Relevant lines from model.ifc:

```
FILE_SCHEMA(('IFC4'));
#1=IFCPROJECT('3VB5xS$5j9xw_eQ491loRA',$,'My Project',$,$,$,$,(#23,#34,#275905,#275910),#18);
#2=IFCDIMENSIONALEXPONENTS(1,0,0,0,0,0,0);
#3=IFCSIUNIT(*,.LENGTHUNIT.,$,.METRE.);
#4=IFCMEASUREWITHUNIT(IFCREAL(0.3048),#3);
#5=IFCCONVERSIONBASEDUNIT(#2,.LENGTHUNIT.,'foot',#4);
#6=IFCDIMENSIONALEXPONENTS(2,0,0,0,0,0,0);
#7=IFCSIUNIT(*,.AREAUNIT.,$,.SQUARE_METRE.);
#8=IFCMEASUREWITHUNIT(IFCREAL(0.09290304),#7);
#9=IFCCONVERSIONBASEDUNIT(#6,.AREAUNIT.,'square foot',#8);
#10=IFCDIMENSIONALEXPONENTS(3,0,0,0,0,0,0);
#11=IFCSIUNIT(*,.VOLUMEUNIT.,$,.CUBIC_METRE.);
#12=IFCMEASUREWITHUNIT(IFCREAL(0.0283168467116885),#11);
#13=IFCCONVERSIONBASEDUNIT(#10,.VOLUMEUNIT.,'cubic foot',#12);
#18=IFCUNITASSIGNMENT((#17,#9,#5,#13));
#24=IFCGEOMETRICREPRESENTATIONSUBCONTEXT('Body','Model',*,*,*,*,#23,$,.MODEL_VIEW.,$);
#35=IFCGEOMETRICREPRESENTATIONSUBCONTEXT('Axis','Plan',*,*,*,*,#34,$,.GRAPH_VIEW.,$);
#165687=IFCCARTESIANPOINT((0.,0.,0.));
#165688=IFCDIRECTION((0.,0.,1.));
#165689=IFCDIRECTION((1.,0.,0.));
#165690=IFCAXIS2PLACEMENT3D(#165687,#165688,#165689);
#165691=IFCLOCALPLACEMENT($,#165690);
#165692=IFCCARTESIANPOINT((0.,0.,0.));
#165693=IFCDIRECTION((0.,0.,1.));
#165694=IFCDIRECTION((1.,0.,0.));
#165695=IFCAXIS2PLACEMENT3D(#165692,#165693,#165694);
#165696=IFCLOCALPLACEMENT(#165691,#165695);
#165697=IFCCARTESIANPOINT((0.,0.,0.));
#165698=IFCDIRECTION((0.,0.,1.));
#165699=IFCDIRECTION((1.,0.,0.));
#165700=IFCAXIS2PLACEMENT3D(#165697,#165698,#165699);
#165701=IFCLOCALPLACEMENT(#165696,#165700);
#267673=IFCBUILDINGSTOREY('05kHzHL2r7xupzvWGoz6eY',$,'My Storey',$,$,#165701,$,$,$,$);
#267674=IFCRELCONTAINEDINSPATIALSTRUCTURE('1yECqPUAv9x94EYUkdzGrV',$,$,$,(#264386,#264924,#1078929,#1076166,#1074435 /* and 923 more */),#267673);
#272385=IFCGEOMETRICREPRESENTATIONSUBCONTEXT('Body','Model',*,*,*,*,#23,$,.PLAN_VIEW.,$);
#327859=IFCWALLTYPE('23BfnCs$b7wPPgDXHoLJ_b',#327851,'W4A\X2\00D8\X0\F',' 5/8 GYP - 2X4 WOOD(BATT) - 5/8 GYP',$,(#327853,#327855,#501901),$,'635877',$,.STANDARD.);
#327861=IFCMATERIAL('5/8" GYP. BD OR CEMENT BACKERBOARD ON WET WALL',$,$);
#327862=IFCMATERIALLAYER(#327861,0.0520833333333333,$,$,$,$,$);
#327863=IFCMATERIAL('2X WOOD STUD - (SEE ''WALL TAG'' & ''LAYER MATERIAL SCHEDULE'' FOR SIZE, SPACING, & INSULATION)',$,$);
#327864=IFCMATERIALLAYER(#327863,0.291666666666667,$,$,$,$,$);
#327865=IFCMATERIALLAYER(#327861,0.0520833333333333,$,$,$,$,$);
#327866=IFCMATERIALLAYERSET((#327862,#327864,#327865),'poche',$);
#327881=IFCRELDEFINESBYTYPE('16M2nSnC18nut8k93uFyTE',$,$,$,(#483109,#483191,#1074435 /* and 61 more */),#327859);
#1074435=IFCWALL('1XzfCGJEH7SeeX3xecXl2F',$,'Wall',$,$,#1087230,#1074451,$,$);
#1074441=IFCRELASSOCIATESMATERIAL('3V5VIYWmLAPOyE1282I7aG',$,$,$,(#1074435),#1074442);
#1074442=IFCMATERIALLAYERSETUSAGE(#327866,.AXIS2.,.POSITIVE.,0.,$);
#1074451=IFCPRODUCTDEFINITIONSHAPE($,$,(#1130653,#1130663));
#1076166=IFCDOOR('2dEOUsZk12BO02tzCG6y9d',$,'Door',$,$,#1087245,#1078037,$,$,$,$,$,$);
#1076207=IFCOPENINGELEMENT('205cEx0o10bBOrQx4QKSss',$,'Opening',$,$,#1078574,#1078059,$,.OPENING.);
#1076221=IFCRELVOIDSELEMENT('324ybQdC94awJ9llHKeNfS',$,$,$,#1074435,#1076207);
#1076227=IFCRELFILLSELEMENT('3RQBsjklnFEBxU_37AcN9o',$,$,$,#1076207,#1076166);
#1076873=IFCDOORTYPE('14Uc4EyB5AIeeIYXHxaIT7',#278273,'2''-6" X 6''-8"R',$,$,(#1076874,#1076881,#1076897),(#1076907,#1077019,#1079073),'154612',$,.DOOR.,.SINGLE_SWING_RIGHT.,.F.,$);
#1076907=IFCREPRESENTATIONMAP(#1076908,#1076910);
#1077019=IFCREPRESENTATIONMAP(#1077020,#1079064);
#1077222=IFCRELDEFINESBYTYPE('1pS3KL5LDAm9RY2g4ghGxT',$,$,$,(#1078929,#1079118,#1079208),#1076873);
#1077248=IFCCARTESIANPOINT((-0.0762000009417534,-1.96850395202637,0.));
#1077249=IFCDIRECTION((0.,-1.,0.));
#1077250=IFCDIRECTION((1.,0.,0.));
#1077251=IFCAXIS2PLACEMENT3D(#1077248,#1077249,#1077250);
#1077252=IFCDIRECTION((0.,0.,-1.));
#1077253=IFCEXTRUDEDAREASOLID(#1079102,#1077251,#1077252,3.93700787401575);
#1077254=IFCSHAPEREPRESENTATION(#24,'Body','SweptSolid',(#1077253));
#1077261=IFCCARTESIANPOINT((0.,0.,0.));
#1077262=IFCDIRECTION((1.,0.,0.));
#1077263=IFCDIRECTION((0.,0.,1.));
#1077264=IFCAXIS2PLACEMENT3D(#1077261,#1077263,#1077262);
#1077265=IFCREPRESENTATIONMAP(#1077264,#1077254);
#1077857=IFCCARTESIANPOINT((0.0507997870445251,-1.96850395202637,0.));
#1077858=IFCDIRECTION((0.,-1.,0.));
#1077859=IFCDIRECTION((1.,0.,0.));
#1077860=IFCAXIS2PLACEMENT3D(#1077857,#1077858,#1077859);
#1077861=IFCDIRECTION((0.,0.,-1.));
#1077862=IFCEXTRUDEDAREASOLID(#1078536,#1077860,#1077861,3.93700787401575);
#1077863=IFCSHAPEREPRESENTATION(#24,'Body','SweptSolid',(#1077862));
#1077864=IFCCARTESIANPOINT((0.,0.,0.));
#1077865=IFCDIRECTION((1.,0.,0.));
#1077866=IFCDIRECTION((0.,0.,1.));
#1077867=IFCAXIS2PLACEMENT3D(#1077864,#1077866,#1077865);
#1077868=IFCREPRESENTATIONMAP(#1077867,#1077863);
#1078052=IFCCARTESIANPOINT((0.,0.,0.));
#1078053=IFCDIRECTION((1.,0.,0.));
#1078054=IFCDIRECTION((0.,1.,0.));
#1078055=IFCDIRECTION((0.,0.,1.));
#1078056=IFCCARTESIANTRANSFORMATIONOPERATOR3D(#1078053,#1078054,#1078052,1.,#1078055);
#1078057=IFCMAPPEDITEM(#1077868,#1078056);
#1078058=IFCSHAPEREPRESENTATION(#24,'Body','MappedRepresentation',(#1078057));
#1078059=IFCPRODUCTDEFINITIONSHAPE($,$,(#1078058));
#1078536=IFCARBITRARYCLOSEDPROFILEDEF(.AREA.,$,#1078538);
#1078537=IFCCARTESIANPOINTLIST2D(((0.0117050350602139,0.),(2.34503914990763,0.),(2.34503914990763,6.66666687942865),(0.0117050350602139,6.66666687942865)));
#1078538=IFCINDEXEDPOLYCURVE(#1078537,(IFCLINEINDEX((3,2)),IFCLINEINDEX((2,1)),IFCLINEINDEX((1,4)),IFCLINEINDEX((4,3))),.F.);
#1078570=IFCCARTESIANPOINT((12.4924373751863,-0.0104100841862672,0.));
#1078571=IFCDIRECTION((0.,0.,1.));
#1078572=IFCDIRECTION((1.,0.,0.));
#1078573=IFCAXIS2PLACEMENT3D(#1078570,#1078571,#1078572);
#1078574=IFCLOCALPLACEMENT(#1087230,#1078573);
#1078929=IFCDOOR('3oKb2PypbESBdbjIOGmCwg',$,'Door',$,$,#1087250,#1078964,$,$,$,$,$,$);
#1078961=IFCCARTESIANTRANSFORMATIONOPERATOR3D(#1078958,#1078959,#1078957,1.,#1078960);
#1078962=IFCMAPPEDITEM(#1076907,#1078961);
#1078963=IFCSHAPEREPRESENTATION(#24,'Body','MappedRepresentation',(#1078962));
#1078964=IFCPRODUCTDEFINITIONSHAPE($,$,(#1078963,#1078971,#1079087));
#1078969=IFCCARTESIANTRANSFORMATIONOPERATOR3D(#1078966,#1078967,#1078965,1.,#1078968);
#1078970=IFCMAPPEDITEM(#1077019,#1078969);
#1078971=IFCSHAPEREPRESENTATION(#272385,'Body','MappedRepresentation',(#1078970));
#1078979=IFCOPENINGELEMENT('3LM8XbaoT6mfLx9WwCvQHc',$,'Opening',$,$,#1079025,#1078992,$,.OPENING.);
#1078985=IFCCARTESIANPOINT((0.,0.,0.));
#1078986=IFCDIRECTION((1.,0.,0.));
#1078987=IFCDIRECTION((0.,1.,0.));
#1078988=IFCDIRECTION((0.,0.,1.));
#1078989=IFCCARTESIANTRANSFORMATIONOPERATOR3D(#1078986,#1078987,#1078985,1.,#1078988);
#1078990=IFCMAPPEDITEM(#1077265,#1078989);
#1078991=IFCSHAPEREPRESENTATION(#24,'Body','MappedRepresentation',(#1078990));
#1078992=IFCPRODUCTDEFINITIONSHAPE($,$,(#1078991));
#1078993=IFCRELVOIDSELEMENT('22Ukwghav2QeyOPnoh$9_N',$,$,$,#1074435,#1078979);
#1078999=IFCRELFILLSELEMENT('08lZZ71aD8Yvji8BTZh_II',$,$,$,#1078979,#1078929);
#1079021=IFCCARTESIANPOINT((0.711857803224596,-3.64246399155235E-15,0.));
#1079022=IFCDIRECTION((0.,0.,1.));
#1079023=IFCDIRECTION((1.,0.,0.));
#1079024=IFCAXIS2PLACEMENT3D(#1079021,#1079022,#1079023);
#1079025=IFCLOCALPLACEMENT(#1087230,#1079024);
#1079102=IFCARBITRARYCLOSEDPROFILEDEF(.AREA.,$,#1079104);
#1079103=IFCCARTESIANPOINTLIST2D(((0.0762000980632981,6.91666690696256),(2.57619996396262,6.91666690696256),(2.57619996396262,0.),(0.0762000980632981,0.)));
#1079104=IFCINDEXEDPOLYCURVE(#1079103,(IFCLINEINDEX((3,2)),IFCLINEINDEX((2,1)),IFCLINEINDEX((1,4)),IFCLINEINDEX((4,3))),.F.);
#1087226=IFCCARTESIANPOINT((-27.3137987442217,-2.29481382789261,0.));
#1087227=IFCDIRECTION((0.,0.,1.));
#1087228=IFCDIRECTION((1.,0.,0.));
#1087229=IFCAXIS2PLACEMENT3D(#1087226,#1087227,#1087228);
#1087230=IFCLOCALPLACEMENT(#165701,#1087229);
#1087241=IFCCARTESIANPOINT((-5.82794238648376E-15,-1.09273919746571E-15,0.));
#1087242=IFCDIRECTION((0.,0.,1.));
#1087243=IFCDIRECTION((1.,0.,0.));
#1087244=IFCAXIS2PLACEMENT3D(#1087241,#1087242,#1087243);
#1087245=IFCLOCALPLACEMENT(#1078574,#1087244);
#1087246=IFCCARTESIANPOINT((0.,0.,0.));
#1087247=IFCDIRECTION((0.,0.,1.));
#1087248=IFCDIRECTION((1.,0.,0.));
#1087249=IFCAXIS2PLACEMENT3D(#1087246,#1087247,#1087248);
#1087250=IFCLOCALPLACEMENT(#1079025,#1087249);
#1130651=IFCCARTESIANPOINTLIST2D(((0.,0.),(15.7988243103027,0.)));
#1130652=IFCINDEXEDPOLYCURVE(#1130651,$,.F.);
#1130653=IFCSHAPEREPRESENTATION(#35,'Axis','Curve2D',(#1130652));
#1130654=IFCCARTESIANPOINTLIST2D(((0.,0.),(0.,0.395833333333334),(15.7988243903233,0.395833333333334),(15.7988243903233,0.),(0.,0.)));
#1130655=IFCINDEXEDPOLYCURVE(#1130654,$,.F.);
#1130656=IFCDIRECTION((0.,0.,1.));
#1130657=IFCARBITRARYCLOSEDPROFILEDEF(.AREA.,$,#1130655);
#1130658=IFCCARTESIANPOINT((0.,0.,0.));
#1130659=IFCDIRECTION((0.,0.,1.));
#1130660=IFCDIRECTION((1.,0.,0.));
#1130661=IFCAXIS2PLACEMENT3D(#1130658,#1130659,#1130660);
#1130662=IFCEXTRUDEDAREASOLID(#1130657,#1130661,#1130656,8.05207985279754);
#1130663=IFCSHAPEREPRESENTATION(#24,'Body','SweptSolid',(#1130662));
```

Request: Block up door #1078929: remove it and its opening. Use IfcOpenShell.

```python
import ifcopenshell
import ifcopenshell.api.feature
import ifcopenshell.api.root
import ifcopenshell.geom
import ifcopenshell.util.shape

model = ifcopenshell.open("model.ifc")
settings = ifcopenshell.geom.settings()


def volume(element):
    """Net volume in cubic metres, openings subtracted."""
    shape = ifcopenshell.geom.create_shape(settings, element)
    return ifcopenshell.util.shape.get_volume(shape.geometry)


door = model.by_guid("3oKb2PypbESBdbjIOGmCwg")
opening = door.FillsVoids[0].RelatingOpeningElement
wall = opening.VoidsElements[0].RelatingBuildingElement
before = volume(wall)

ifcopenshell.api.root.remove_product(model, product=door)
ifcopenshell.api.feature.remove_feature(model, feature=opening)

after = volume(wall)

print(f"wall volume {before:.3f} -> {after:.3f} m3")

model.write("model_v2.ifc")
```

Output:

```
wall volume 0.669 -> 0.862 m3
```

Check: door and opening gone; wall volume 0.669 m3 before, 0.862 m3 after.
